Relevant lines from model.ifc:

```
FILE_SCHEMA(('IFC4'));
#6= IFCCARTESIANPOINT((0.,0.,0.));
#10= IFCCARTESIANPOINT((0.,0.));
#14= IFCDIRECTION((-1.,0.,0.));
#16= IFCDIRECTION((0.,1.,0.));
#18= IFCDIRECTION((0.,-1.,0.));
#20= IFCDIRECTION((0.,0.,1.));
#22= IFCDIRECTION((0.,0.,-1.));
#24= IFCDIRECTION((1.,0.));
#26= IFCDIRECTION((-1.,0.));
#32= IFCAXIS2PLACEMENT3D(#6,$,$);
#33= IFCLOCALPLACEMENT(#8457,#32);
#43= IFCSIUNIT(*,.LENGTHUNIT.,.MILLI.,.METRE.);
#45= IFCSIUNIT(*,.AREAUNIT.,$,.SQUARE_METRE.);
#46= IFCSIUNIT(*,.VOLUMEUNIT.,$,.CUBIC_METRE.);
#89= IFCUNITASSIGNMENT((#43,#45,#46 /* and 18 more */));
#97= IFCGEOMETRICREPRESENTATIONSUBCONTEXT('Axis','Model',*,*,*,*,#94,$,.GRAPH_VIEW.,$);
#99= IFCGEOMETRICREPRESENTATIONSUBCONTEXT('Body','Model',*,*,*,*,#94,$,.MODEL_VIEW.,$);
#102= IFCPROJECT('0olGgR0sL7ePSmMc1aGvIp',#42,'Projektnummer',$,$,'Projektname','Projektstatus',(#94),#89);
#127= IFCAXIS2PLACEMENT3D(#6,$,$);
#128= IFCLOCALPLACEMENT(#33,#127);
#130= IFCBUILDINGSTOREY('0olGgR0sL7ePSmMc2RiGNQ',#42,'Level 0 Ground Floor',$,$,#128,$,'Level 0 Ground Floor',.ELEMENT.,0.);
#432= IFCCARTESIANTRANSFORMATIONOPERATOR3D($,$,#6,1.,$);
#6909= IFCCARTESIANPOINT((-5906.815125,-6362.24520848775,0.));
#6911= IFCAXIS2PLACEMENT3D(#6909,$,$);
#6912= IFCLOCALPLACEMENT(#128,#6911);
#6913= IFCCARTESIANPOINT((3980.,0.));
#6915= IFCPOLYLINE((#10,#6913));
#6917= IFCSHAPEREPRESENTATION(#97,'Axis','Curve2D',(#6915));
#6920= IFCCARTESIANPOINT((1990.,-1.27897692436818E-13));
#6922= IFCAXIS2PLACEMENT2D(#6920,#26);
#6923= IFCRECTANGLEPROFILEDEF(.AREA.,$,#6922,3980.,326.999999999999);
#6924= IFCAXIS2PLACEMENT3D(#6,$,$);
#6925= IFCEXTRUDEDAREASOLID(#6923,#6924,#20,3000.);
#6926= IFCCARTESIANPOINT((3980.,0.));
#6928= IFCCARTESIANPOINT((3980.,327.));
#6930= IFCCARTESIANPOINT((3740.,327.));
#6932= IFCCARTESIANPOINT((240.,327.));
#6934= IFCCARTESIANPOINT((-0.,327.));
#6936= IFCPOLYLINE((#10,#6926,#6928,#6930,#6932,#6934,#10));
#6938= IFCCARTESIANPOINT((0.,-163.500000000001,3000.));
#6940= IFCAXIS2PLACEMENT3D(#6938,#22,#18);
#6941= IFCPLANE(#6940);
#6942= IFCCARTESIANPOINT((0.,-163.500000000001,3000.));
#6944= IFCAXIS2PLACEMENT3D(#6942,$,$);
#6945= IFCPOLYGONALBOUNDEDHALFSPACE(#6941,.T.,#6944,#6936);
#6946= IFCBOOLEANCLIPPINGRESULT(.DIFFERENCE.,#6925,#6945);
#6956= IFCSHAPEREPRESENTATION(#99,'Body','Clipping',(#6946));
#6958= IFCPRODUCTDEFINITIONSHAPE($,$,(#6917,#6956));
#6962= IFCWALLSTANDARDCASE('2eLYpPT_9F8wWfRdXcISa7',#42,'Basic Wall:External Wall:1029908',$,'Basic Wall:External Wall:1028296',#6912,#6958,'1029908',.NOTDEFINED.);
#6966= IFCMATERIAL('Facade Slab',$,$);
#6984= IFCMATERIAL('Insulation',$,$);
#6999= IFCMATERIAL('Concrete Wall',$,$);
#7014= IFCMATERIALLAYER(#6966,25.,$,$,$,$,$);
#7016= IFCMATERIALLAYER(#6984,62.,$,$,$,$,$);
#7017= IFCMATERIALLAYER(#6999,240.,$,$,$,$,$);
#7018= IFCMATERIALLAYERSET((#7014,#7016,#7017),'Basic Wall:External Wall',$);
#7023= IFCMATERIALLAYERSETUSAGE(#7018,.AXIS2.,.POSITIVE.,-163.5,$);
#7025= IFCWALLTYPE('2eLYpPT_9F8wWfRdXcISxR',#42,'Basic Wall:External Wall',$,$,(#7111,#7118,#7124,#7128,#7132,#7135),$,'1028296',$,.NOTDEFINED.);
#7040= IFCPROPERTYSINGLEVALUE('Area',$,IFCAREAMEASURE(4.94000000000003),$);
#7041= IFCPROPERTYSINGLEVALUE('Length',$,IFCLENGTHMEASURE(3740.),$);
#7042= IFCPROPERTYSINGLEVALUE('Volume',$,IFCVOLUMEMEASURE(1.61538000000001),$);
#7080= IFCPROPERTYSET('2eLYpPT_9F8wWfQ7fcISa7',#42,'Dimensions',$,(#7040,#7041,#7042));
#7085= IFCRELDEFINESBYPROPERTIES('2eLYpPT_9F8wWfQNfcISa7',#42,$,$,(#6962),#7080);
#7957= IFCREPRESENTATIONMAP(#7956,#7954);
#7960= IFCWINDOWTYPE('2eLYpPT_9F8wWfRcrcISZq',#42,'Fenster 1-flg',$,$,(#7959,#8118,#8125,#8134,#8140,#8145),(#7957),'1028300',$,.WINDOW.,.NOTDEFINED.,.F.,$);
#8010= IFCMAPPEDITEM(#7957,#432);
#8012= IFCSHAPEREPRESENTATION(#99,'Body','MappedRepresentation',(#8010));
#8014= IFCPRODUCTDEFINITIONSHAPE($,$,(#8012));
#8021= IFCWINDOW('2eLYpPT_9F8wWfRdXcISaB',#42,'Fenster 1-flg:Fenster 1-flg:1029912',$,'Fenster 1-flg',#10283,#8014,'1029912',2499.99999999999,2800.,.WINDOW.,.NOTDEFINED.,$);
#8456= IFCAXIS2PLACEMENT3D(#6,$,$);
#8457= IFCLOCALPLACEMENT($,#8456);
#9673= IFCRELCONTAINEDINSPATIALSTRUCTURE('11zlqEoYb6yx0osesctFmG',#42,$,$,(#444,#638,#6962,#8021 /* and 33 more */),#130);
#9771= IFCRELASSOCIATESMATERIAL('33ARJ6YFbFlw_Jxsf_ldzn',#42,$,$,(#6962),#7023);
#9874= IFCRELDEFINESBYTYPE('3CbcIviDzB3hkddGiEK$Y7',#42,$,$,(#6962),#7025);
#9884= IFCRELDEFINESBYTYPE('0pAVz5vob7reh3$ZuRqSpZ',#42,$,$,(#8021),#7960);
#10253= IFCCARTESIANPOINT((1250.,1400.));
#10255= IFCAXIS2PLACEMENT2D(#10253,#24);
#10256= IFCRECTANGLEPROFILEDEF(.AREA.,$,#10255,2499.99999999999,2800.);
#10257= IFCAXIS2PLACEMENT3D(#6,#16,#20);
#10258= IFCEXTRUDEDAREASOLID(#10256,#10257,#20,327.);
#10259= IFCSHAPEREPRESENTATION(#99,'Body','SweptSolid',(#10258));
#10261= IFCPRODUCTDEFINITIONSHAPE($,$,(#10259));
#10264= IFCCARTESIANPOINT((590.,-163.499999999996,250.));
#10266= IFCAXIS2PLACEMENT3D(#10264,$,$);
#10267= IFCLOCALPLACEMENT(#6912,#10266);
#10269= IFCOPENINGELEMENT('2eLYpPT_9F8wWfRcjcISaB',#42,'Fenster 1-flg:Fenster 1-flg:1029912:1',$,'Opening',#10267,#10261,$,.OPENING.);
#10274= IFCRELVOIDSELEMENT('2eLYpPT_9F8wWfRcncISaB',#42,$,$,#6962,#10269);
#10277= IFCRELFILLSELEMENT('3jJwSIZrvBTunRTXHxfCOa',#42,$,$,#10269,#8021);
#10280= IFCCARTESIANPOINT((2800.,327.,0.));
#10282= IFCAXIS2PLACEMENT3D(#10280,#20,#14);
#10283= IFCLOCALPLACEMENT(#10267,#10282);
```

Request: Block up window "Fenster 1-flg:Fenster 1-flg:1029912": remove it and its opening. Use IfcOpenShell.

```python
import ifcopenshell
import ifcopenshell.api.feature
import ifcopenshell.api.pset
import ifcopenshell.api.root
import ifcopenshell.geom
import ifcopenshell.util.element
import ifcopenshell.util.shape
import ifcopenshell.util.unit

model = ifcopenshell.open("model.ifc")
area_scale = ifcopenshell.util.unit.calculate_unit_scale(model, "AREAUNIT")
volume_scale = ifcopenshell.util.unit.calculate_unit_scale(model, "VOLUMEUNIT")
settings = ifcopenshell.geom.settings()


def volume(element):
    """Net volume in cubic metres, openings subtracted."""
    shape = ifcopenshell.geom.create_shape(settings, element)
    return ifcopenshell.util.shape.get_volume(shape.geometry)


window = model.by_guid("2eLYpPT_9F8wWfRdXcISaB")
opening = window.FillsVoids[0].RelatingOpeningElement
wall = opening.VoidsElements[0].RelatingBuildingElement
before = volume(wall)

ifcopenshell.api.root.remove_product(model, product=window)
ifcopenshell.api.feature.remove_feature(model, feature=opening)

after = volume(wall)
thickness = 0.327  # wall thickness in metres

# Update the wall's stored quantities.
pset = model.by_id(ifcopenshell.util.element.get_pset(wall, "Dimensions", should_inherit=False)["id"])
ifcopenshell.api.pset.edit_pset(model, pset=pset, properties={
    "Area": model.create_entity("IfcAreaMeasure", after / thickness / area_scale),
    "Volume": model.create_entity("IfcVolumeMeasure", after / volume_scale),
})

print(f"wall volume {before:.3f} -> {after:.3f} m3")

model.write("model-out.ifc")
```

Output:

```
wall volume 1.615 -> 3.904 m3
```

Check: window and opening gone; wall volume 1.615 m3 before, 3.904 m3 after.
